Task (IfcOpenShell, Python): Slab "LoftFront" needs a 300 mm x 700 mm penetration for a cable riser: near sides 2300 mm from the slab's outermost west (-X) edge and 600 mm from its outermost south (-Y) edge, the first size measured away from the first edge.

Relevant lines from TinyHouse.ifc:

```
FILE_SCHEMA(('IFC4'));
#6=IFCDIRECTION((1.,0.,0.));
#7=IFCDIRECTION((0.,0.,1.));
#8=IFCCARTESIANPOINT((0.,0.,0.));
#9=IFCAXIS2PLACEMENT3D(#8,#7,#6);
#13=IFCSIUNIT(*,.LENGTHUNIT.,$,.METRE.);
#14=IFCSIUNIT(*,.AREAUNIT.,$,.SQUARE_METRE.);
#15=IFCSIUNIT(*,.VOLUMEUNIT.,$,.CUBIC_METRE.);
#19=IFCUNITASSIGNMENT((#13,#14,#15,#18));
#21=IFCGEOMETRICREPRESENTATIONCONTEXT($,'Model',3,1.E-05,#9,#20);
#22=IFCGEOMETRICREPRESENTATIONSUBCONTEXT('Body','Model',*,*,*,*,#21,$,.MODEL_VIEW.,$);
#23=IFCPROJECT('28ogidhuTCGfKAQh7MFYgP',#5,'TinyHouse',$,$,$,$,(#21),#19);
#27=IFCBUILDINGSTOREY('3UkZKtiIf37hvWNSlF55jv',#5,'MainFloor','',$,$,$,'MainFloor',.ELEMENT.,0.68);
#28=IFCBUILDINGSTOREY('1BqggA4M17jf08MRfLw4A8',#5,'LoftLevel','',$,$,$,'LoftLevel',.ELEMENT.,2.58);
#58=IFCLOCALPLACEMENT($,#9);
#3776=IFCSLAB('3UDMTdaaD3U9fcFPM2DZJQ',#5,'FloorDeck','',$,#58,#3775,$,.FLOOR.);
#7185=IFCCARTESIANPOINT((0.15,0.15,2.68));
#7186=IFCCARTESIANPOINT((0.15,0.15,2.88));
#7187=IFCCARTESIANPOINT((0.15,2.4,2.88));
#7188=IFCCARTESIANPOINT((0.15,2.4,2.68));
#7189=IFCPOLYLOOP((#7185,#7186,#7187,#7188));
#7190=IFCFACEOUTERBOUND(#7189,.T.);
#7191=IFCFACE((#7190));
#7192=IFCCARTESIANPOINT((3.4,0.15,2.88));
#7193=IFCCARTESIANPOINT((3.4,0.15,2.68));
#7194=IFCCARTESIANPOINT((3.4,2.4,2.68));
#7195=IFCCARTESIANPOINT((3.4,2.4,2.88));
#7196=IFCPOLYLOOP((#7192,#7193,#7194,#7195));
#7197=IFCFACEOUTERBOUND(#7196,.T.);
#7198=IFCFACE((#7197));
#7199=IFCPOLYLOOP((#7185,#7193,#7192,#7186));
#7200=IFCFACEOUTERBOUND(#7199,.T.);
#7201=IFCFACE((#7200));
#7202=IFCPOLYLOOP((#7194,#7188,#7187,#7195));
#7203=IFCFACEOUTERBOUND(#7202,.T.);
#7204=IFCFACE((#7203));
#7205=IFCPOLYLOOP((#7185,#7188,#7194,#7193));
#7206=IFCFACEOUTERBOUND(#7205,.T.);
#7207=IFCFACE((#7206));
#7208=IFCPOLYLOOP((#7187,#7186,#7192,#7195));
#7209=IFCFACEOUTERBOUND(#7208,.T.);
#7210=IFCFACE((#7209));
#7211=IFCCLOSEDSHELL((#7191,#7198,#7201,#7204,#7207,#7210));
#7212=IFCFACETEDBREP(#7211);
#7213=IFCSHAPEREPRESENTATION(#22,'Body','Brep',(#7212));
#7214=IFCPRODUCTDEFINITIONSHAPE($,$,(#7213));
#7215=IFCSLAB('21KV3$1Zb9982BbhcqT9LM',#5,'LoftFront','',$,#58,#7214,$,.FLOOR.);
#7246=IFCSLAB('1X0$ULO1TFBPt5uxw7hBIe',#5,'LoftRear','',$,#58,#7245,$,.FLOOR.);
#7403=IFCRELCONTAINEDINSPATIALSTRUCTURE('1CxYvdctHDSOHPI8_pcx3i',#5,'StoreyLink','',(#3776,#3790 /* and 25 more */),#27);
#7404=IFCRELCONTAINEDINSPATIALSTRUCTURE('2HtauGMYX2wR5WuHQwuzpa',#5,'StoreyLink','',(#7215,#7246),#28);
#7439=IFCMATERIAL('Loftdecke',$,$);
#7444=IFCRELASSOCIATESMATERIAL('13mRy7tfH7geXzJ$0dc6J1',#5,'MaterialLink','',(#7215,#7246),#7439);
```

```python
import numpy as np
import ifcopenshell
import ifcopenshell.api.feature
import ifcopenshell.api.geometry
import ifcopenshell.api.root
import ifcopenshell.geom
import ifcopenshell.util.placement
import ifcopenshell.util.representation
import ifcopenshell.util.shape
import ifcopenshell.util.unit

model = ifcopenshell.open("TinyHouse.ifc")
unit_scale = ifcopenshell.util.unit.calculate_unit_scale(model)
settings = ifcopenshell.geom.settings()


def volume(element):
    """Net volume in cubic metres, openings subtracted."""
    shape = ifcopenshell.geom.create_shape(settings, element)
    return ifcopenshell.util.shape.get_volume(shape.geometry)


slab = model.by_guid("21KV3$1Zb9982BbhcqT9LM")
before = volume(slab)

# Extent in the slab's own axes, in metres. The edges named are its -X and -Y sides.
slab_shape = ifcopenshell.geom.create_shape(settings, slab)
vertices = ifcopenshell.util.shape.get_vertices(slab_shape.geometry)
x_min, y_min, bottom = vertices.min(axis=0)
top = vertices[:, 2].max()

opening = ifcopenshell.api.root.create_entity(model, ifc_class="IfcOpeningElement", name="Cable riser opening", predefined_type="OPENING")
context = ifcopenshell.util.representation.get_context(model, "Model", "Body", "MODEL_VIEW")
width, depth = 0.3, 0.7
outline = [(0.0, 0.0), (width, 0.0), (width, depth), (0.0, depth), (0.0, 0.0)]
# Overshoot both faces by 50 mm so the cut is clean.
shape = ifcopenshell.api.geometry.add_slab_representation(
    model, context=context, depth=top - bottom + 0.1, polyline=outline
)
ifcopenshell.api.geometry.assign_representation(model, product=opening, representation=shape)

matrix = ifcopenshell.util.placement.get_local_placement(slab.ObjectPlacement)
matrix[:, 3] = matrix @ np.append(np.array([x_min + 2.3, y_min + 0.6, bottom - 0.05]) / unit_scale, 1.0)
ifcopenshell.api.geometry.edit_object_placement(model, product=opening, matrix=matrix, is_si=False)
ifcopenshell.api.feature.add_feature(model, feature=opening, element=slab)

after = volume(slab)

print(f"slab volume {before:.3f} -> {after:.3f} m3")

model.write("TinyHouse_rev.ifc")
```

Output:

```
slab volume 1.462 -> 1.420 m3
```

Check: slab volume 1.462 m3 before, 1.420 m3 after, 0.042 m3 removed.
